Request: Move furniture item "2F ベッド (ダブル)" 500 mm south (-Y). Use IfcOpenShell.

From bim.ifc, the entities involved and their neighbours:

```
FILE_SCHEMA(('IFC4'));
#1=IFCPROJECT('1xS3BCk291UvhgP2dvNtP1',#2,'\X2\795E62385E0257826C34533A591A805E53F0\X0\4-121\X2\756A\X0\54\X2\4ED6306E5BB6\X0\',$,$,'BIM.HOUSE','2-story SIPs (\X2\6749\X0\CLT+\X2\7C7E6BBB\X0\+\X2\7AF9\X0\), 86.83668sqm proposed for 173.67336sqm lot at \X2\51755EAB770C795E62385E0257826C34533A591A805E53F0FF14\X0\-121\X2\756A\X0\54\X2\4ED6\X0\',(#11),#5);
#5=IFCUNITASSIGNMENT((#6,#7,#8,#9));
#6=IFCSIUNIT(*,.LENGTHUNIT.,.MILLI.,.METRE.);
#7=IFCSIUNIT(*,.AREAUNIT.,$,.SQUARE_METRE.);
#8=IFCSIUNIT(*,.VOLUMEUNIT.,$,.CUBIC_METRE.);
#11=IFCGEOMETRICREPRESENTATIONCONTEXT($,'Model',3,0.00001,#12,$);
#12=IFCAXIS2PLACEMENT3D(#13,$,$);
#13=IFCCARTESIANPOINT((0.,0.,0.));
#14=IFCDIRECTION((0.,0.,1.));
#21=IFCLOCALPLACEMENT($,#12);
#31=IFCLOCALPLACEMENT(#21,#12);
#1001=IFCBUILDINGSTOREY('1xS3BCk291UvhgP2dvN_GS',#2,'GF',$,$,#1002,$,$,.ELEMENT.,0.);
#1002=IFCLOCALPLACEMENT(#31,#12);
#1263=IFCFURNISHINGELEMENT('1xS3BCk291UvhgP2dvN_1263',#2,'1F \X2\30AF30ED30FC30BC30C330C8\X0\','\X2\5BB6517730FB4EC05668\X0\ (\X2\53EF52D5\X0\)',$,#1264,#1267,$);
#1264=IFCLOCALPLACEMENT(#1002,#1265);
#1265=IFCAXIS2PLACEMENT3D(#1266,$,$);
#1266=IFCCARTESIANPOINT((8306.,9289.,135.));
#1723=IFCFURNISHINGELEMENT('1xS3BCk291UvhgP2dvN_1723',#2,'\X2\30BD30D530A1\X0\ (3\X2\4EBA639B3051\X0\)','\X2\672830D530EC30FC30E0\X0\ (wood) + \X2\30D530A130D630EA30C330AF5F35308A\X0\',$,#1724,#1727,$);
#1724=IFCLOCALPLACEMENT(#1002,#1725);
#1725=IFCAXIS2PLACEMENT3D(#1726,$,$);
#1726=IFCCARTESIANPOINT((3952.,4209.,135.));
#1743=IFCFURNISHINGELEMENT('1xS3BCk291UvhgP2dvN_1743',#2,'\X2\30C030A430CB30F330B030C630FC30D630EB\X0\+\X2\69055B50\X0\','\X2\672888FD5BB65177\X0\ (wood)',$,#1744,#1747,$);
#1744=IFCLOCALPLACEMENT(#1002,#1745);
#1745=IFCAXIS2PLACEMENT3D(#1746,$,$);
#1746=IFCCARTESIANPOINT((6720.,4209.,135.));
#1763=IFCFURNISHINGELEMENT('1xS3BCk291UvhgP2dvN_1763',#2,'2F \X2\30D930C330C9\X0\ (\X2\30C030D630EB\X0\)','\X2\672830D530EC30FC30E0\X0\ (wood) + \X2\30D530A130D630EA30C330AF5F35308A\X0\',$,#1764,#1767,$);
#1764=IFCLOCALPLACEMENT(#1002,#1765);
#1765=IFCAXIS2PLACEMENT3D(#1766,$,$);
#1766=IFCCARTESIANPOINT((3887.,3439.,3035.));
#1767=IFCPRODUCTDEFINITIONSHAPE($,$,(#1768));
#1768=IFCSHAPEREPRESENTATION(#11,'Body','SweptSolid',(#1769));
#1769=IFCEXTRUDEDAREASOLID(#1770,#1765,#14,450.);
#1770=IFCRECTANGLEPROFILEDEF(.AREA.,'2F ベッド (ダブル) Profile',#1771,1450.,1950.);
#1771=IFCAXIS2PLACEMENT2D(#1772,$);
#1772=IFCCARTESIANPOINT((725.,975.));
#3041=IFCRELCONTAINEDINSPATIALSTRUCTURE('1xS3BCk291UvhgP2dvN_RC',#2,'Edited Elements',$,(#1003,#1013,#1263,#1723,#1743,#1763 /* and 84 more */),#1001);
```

```python
import ifcopenshell
import ifcopenshell.api.geometry
import ifcopenshell.util.placement

model = ifcopenshell.open("bim.ifc")

item = model.by_guid("1xS3BCk291UvhgP2dvN_1763")
matrix = ifcopenshell.util.placement.get_local_placement(item.ObjectPlacement)
matrix[1, 3] -= 500.0
ifcopenshell.api.geometry.edit_object_placement(model, product=item, matrix=matrix, is_si=False)

print(ifcopenshell.util.placement.get_local_placement(item.ObjectPlacement).round(3) + 0.0)

model.write("bim-out.ifc")
```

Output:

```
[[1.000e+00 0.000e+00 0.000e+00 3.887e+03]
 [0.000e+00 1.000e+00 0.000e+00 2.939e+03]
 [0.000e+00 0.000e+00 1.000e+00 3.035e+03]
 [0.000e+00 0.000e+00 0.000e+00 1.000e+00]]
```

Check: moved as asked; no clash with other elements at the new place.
